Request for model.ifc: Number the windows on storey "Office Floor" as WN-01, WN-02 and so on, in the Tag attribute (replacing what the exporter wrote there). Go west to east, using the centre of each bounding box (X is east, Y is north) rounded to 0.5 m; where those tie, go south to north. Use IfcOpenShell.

First a look at what the model holds.

```python
import ifcopenshell
import ifcopenshell.util.element
import ifcopenshell.util.placement

model = ifcopenshell.open("model.ifc")
print(model.schema)
storey = next(s for s in model.by_type("IfcBuildingStorey") if s.Name == "Office Floor")
windows = [e for e in ifcopenshell.util.element.get_decomposition(storey) if e.is_a("IfcWindow")]
for e in sorted(windows, key=lambda e: e.id()):
    origin = ifcopenshell.util.placement.get_local_placement(e.ObjectPlacement)[:3, 3]
    print(e.id(), e.Tag, e.Name, origin.round(2) + 0.0, sep=" | ")
```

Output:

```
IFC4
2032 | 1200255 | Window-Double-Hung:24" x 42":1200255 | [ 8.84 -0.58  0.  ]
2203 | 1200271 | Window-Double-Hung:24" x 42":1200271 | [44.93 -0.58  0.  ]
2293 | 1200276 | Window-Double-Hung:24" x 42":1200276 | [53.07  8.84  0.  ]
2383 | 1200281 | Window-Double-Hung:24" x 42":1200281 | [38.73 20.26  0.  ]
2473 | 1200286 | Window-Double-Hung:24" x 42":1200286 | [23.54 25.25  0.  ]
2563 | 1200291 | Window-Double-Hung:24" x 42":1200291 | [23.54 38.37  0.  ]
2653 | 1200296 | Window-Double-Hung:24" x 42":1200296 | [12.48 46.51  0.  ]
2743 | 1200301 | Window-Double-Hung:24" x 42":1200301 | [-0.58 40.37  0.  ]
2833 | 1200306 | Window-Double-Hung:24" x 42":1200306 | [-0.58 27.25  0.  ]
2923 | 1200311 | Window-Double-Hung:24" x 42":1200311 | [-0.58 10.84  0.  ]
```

```python
import ifcopenshell
import ifcopenshell.geom
import ifcopenshell.util.element
import ifcopenshell.util.shape

model = ifcopenshell.open("model.ifc")
settings = ifcopenshell.geom.settings()
settings.set("use-world-coords", True)


def centre(element):
    shape = ifcopenshell.geom.create_shape(settings, element)
    return ifcopenshell.util.shape.get_bbox_centroid(shape.geometry)


storey = next(s for s in model.by_type("IfcBuildingStorey") if s.Name == "Office Floor")
windows = [e for e in ifcopenshell.util.element.get_decomposition(storey) if e.is_a("IfcWindow")]

# Insertion points can sit at a corner or the storey origin, so sort by the geometry (in metres).
centres = {e: centre(e) for e in windows}
windows.sort(key=lambda e: (round(centres[e][0] / 0.5), centres[e][1]))

for i, e in enumerate(windows, start=1):
    number = f"WN-{i:02d}"
    e.Tag = number
    print(e.id(), number)

model.write("model_updated.ifc")
```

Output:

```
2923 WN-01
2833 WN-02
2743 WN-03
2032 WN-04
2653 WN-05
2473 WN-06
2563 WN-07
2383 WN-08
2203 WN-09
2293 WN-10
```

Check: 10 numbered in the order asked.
